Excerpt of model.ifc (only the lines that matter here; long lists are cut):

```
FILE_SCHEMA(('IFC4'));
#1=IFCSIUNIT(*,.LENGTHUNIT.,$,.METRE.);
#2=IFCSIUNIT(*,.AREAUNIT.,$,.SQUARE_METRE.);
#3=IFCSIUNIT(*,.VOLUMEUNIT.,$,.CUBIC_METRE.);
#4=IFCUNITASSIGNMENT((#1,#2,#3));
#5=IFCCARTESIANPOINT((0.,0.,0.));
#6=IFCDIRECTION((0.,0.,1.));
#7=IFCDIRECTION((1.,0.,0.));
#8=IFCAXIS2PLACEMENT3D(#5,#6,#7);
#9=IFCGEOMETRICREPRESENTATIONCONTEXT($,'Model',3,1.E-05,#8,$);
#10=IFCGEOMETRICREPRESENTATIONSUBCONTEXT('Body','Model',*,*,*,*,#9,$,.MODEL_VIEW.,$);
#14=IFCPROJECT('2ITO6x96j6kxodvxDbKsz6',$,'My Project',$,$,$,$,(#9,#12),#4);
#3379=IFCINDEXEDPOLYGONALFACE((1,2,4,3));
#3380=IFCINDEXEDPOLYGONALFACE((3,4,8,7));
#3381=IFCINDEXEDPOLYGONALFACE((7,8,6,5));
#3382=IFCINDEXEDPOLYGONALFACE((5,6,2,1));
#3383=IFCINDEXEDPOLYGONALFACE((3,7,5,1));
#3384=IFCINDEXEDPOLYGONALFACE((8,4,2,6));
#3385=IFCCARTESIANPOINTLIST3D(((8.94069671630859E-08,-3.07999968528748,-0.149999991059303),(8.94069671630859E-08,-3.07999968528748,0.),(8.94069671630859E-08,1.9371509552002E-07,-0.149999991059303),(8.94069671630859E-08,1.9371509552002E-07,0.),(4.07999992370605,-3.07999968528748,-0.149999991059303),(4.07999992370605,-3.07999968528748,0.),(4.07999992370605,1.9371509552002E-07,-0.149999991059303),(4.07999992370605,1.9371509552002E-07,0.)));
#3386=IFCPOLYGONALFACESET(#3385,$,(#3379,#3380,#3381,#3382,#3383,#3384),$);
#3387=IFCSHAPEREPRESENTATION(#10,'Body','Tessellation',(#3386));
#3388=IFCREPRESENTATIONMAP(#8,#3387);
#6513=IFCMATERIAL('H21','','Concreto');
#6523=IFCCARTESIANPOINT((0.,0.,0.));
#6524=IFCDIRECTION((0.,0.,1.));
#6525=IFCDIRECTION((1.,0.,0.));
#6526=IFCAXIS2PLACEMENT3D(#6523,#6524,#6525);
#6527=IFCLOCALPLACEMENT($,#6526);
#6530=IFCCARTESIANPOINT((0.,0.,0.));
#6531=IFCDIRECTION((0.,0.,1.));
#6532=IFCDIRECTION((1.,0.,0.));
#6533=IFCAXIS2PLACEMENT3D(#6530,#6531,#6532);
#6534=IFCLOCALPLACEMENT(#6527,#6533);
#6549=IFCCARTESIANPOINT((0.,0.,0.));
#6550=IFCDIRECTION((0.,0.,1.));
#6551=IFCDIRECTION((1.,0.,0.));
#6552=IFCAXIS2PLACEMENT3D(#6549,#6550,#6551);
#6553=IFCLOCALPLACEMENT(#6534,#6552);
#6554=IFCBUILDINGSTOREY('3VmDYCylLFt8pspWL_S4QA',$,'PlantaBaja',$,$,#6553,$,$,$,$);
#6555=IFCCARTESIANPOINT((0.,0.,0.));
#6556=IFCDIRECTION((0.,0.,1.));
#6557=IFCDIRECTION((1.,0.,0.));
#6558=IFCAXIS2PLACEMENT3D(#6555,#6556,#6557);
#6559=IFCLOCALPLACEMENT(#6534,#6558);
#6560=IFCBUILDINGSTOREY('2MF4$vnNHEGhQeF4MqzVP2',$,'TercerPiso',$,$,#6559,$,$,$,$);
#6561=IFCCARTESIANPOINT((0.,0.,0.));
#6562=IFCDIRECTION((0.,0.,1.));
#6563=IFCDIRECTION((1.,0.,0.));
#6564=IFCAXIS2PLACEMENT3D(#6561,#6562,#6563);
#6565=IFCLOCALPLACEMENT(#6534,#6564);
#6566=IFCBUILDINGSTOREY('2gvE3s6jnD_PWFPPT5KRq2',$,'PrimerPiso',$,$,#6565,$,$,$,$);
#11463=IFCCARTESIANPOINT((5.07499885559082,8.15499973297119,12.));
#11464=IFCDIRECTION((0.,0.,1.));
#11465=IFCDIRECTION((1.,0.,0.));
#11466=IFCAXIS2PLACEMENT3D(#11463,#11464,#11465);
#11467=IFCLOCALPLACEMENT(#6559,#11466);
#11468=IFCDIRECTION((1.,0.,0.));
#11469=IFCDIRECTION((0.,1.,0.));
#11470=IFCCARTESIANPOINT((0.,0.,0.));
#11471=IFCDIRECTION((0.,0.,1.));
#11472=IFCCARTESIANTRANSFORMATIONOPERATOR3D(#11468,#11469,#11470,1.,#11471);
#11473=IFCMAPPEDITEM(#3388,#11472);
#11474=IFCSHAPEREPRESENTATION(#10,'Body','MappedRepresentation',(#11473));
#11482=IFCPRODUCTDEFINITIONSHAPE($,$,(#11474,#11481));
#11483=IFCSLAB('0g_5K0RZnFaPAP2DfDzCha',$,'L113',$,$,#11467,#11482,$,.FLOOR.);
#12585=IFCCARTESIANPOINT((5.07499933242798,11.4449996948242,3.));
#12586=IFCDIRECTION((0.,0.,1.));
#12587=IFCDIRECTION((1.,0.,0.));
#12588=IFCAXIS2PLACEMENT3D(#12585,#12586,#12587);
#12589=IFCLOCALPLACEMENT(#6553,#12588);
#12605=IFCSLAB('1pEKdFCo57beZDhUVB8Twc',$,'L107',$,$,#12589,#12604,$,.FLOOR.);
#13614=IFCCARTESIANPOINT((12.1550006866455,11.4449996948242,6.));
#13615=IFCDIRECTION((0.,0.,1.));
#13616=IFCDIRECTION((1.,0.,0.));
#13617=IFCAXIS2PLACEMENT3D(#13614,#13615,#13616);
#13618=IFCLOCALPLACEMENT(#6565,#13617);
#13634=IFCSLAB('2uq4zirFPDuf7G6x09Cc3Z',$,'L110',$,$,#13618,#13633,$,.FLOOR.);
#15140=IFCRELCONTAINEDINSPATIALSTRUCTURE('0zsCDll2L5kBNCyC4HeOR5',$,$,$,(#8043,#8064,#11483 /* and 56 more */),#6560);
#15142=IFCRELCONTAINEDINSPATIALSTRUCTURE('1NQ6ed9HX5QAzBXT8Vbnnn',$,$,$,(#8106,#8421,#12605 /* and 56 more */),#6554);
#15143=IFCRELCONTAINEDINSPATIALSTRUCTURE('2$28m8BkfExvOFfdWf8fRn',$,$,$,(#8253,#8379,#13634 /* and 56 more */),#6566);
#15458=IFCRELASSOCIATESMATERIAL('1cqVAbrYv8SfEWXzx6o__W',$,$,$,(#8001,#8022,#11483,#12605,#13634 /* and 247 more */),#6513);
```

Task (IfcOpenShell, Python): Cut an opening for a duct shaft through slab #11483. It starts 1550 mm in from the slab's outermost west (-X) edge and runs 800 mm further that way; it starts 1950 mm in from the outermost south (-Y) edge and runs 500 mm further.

```python
import numpy as np
import ifcopenshell
import ifcopenshell.api.feature
import ifcopenshell.api.geometry
import ifcopenshell.api.root
import ifcopenshell.geom
import ifcopenshell.util.placement
import ifcopenshell.util.representation
import ifcopenshell.util.shape
import ifcopenshell.util.unit

model = ifcopenshell.open("model.ifc")
unit_scale = ifcopenshell.util.unit.calculate_unit_scale(model)
settings = ifcopenshell.geom.settings()


def volume(element):
    """Net volume in cubic metres, openings subtracted."""
    shape = ifcopenshell.geom.create_shape(settings, element)
    return ifcopenshell.util.shape.get_volume(shape.geometry)


slab = model.by_id(11483)
before = volume(slab)

# Extent in the slab's own axes, in metres. The edges named are its -X and -Y sides.
slab_shape = ifcopenshell.geom.create_shape(settings, slab)
vertices = ifcopenshell.util.shape.get_vertices(slab_shape.geometry)
x_min, y_min, bottom = vertices.min(axis=0)
top = vertices[:, 2].max()

opening = ifcopenshell.api.root.create_entity(model, ifc_class="IfcOpeningElement", name="Duct shaft opening", predefined_type="OPENING")
context = ifcopenshell.util.representation.get_context(model, "Model", "Body", "MODEL_VIEW")
width, depth = 0.8, 0.5
outline = [(0.0, 0.0), (width, 0.0), (width, depth), (0.0, depth), (0.0, 0.0)]
# Overshoot both faces by 50 mm so the cut is clean.
shape = ifcopenshell.api.geometry.add_slab_representation(
    model, context=context, depth=top - bottom + 0.1, polyline=outline
)
ifcopenshell.api.geometry.assign_representation(model, product=opening, representation=shape)

matrix = ifcopenshell.util.placement.get_local_placement(slab.ObjectPlacement)
matrix[:, 3] = matrix @ np.append(np.array([x_min + 1.55, y_min + 1.95, bottom - 0.05]) / unit_scale, 1.0)
ifcopenshell.api.geometry.edit_object_placement(model, product=opening, matrix=matrix, is_si=False)
ifcopenshell.api.feature.add_feature(model, feature=opening, element=slab)

after = volume(slab)

print(f"slab volume {before:.3f} -> {after:.3f} m3")

model.write("model_edited.ifc")
```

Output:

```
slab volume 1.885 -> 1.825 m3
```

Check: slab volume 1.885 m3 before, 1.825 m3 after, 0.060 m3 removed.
